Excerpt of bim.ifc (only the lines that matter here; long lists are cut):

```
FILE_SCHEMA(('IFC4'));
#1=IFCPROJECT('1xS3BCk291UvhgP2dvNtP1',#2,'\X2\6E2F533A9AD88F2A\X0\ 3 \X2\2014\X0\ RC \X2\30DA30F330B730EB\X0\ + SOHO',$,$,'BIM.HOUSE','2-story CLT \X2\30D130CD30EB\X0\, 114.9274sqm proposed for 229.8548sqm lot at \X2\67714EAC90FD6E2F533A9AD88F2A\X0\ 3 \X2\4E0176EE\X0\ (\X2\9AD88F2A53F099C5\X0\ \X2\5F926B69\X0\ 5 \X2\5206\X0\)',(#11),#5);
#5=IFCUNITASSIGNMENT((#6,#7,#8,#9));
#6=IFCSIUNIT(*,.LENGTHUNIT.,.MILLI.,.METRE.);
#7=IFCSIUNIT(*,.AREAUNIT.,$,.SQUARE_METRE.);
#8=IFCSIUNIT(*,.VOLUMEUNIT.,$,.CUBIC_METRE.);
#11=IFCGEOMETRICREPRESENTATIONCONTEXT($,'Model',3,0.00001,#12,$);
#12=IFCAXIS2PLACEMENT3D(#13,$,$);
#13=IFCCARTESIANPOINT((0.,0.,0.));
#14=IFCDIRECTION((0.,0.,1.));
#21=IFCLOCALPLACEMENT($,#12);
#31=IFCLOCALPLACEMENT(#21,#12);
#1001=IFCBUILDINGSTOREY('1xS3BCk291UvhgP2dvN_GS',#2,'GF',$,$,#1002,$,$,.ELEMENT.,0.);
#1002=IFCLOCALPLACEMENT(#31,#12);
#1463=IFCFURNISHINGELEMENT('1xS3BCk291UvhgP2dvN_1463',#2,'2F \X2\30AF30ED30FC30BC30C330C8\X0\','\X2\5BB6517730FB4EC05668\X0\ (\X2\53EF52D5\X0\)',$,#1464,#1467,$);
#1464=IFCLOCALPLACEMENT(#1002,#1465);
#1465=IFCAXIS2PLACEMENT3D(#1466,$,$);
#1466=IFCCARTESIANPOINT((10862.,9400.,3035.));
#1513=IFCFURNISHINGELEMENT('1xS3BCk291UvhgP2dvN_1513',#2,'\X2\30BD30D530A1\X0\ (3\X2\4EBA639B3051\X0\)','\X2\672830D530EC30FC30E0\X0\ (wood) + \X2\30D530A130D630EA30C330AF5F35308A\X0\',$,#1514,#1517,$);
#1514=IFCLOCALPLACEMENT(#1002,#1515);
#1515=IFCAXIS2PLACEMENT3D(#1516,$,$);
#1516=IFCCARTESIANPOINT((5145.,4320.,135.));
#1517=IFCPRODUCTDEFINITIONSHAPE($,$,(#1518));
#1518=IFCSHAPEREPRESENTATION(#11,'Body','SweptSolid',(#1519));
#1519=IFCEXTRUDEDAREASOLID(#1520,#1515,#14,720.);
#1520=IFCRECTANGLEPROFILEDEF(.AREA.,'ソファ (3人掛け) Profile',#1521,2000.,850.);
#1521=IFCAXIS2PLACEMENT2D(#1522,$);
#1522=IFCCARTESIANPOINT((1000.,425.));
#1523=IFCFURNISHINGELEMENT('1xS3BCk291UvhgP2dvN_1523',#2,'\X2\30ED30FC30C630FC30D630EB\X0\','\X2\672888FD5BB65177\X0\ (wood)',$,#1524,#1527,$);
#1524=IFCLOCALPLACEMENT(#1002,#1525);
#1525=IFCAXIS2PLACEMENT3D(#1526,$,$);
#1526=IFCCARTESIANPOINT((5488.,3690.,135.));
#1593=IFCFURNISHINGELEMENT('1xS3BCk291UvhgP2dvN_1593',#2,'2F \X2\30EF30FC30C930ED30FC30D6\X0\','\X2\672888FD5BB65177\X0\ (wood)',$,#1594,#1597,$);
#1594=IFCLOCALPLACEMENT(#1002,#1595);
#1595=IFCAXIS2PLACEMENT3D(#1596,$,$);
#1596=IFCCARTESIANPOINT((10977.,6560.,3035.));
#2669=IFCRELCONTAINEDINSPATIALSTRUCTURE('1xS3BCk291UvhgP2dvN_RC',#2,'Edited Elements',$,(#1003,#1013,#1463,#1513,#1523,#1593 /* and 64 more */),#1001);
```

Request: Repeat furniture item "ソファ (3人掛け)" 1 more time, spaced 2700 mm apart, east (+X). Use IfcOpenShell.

```python
import numpy as np
import ifcopenshell
import ifcopenshell.api.geometry
import ifcopenshell.api.root
import ifcopenshell.util.element
import ifcopenshell.util.placement
import ifcopenshell.util.unit

model = ifcopenshell.open("bim.ifc")
unit_scale = ifcopenshell.util.unit.calculate_unit_scale(model)


def reuse_history(source, copy):
    """copy_class also copies each property set's owner history, people and application; keep the originals."""
    for rel in copy.IsDefinedBy:
        if rel.is_a("IfcRelDefinesByProperties") and (history := rel.RelatingPropertyDefinition.OwnerHistory):
            rel.RelatingPropertyDefinition.OwnerHistory = source.OwnerHistory
            ifcopenshell.util.element.remove_deep2(model, history)


source = model.by_guid("1xS3BCk291UvhgP2dvN_1513")
base = ifcopenshell.util.placement.get_local_placement(source.ObjectPlacement)
step = np.array([1.0, 0.0, 0.0]) * 2.7 / unit_scale

for i in range(1, 2):
    copy = ifcopenshell.api.root.copy_class(model, product=source)
    copy.Representation = ifcopenshell.util.element.copy_deep(
        model, source.Representation, exclude=["IfcGeometricRepresentationContext", "IfcRepresentationMap"]
    )
    reuse_history(source, copy)
    matrix = base.copy()
    matrix[:3, 3] += i * step
    print("added at", matrix[:3, 3].round(3) + 0.0)
    ifcopenshell.api.geometry.edit_object_placement(model, product=copy, matrix=matrix, is_si=False)

model.write("bim_v2.ifc")
```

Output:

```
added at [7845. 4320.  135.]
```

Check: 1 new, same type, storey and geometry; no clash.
